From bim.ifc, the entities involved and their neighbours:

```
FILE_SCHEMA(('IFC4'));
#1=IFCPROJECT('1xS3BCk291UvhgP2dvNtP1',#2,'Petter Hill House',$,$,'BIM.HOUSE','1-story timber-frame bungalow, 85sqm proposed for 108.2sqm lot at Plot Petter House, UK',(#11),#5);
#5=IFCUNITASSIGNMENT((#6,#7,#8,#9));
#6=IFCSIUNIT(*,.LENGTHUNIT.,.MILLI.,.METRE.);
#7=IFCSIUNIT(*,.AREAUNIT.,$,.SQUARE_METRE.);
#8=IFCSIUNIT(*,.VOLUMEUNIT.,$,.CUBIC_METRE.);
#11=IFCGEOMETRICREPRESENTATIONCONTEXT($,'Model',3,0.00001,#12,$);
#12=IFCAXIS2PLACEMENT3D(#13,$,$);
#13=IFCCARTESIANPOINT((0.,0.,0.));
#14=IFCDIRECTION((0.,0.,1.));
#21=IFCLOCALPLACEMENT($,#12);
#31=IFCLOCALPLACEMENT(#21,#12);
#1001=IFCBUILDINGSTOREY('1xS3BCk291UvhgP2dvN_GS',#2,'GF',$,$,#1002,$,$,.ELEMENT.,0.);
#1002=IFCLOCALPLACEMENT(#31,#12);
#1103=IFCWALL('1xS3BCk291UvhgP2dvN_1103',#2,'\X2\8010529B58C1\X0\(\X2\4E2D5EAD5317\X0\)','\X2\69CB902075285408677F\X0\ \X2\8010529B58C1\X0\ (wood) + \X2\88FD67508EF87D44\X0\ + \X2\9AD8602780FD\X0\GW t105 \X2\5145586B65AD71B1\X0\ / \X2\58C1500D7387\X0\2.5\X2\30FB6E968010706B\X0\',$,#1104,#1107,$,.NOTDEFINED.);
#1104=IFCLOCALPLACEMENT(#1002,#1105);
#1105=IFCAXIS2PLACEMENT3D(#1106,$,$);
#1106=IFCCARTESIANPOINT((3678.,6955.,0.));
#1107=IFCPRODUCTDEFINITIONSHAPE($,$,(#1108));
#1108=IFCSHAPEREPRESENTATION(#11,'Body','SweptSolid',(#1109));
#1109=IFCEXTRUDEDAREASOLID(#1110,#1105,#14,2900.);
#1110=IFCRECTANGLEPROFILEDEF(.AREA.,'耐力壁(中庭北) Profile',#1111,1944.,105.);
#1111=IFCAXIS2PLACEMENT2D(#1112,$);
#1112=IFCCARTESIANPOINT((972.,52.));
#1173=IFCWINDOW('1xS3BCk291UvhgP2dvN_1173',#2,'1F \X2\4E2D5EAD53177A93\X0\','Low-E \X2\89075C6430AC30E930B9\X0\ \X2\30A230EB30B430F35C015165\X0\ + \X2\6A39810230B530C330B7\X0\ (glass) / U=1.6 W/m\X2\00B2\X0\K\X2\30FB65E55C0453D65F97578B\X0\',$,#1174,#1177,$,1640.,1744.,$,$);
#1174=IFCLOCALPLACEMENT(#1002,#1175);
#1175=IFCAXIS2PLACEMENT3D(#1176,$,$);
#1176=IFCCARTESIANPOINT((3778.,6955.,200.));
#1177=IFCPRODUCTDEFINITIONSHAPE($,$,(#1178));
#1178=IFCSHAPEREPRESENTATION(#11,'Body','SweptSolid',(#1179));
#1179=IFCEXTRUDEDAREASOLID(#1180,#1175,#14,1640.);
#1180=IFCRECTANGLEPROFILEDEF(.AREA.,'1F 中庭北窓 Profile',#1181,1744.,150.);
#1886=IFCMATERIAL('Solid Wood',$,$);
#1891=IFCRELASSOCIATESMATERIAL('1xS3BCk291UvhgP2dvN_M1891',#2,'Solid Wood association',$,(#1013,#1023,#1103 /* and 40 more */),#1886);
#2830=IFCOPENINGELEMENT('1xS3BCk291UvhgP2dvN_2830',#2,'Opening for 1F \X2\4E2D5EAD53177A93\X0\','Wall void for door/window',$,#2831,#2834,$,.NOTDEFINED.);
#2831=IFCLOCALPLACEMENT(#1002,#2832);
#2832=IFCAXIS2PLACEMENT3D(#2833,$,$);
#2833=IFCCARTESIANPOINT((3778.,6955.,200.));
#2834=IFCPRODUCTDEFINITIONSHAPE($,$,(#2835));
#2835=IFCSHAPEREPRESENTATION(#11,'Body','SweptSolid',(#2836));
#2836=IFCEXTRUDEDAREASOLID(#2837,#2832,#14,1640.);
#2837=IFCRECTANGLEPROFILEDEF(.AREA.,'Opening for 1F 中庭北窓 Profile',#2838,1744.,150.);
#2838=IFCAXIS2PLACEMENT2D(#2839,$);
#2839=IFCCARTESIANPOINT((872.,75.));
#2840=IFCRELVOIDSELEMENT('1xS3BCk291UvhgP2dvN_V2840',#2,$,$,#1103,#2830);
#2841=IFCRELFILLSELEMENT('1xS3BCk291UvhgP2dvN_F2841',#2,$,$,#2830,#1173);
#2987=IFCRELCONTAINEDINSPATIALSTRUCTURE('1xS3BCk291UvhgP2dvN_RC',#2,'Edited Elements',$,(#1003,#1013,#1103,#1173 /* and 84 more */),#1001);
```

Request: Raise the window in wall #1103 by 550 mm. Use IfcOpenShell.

```python
import numpy as np
import ifcopenshell
import ifcopenshell.api.geometry
import ifcopenshell.util.placement
import ifcopenshell.util.unit

model = ifcopenshell.open("bim.ifc")
unit_scale = ifcopenshell.util.unit.calculate_unit_scale(model)

window = model.by_guid("1xS3BCk291UvhgP2dvN_1173")
opening = window.FillsVoids[0].RelatingOpeningElement
dz = 0.55 / unit_scale

shift = np.array([0.0, 0.0, dz])
# The window is not placed relative to its opening, so move both.
for product in (opening, window):
    matrix = ifcopenshell.util.placement.get_local_placement(product.ObjectPlacement)
    matrix[:3, 3] += shift
    ifcopenshell.api.geometry.edit_object_placement(model, product=product, matrix=matrix, is_si=False)

print(f"moved by {dz * unit_scale:+.3f} m")

model.write("bim-out.ifc")
```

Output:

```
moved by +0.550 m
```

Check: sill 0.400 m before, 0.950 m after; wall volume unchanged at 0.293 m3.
